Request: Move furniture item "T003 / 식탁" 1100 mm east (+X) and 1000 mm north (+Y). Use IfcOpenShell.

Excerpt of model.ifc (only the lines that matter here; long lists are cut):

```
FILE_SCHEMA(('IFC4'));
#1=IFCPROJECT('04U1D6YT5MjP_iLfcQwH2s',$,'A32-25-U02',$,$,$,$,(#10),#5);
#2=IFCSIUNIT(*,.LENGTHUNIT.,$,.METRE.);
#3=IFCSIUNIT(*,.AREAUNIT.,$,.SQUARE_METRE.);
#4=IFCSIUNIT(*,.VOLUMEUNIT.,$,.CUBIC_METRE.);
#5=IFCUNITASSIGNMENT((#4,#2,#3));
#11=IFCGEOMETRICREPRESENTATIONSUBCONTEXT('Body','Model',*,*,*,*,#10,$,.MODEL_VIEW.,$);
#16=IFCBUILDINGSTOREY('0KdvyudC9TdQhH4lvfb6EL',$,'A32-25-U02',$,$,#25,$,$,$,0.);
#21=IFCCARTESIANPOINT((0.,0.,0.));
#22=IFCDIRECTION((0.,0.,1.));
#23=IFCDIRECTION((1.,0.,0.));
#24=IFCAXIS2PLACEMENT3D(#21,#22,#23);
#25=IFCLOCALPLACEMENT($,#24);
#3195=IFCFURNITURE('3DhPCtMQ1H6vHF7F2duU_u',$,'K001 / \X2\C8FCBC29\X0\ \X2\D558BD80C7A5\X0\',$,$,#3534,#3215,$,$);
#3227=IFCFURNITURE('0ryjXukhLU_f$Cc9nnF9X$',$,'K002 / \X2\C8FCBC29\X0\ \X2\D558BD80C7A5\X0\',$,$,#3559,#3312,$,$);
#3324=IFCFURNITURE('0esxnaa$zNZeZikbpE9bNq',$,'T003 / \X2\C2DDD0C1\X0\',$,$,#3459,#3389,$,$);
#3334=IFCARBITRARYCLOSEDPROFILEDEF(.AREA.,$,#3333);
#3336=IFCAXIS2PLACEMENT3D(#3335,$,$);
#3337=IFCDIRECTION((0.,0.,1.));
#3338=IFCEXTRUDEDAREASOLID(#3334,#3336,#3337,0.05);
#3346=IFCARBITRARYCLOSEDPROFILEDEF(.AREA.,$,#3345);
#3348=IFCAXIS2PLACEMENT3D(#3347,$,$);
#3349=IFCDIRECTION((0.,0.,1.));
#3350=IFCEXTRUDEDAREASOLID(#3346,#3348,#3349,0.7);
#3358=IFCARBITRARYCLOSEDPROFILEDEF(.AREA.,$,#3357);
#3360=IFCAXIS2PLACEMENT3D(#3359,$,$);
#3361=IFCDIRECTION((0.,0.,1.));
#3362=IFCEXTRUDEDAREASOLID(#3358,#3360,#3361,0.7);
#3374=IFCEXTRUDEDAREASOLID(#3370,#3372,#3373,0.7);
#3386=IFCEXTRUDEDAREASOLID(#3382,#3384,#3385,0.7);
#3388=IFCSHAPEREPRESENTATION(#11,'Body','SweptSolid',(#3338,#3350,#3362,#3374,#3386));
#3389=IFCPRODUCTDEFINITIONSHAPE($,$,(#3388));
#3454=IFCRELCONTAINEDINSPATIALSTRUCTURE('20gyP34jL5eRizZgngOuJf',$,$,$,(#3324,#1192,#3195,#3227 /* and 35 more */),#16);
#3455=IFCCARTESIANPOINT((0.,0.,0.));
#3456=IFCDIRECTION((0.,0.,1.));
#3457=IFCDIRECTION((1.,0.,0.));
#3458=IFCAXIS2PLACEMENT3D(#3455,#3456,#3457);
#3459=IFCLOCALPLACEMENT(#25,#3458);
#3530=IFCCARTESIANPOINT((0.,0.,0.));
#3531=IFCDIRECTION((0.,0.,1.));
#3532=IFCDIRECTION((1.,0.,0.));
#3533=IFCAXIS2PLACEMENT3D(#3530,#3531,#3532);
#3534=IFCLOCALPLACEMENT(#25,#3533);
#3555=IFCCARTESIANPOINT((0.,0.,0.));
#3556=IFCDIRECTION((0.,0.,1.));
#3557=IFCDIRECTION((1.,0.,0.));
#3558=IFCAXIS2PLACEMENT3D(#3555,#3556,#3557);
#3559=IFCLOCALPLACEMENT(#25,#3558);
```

```python
import ifcopenshell
import ifcopenshell.api.geometry
import ifcopenshell.util.placement
import ifcopenshell.util.unit

model = ifcopenshell.open("model.ifc")
unit_scale = ifcopenshell.util.unit.calculate_unit_scale(model)

item = model.by_id(3324)
matrix = ifcopenshell.util.placement.get_local_placement(item.ObjectPlacement)
matrix[0, 3] += 1.1 / unit_scale
matrix[1, 3] += 1 / unit_scale
ifcopenshell.api.geometry.edit_object_placement(model, product=item, matrix=matrix, is_si=False)

print(ifcopenshell.util.placement.get_local_placement(item.ObjectPlacement).round(3) + 0.0)

model.write("model_updated.ifc")
```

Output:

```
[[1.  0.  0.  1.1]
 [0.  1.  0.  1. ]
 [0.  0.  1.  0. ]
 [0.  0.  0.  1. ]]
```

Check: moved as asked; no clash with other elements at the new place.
